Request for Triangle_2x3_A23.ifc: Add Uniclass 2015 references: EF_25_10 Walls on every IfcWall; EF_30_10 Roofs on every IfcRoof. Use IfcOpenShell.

First a look at what the model holds.

```python
import ifcopenshell

model = ifcopenshell.open("Triangle_2x3_A23.ifc")
print(model.schema)
print("classifications:", [c.Name for c in model.by_type("IfcClassification")])
for ifc_class in ("IfcDoor", "IfcRoof", "IfcStair", "IfcWall", "IfcWindow"):
    print(ifc_class, len(model.by_type(ifc_class)))
```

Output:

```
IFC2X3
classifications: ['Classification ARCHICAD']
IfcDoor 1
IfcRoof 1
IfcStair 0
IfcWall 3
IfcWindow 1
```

```python
import ifcopenshell
import ifcopenshell.api.classification

model = ifcopenshell.open("Triangle_2x3_A23.ifc")

# IFC2X3 requires Source and Edition and has no link from the project to the system.
system = model.create_entity("IfcClassification", Source="NBS", Edition="2015", Name="Uniclass 2015")

codes = {
    "IfcWall": ("EF_25_10", "Walls"),
    "IfcRoof": ("EF_30_10", "Roofs"),
}
for ifc_class, (code, name) in codes.items():
    products = model.by_type(ifc_class)
    ifcopenshell.api.classification.add_reference(
        model, products=products, classification=system, identification=code, name=name
    )
    print(code, len(products))

model.write("Triangle_2x3_A23_rev.ifc")
```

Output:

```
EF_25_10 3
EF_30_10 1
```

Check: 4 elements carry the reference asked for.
